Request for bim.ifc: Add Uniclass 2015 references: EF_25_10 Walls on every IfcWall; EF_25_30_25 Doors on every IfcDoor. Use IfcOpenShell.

First a look at what the model holds.

```python
import ifcopenshell

model = ifcopenshell.open("bim.ifc")
print(model.schema)
print("classifications:", [c.Name for c in model.by_type("IfcClassification")])
for ifc_class in ("IfcDoor", "IfcRoof", "IfcStair", "IfcWall", "IfcWindow"):
    print(ifc_class, len(model.by_type(ifc_class)))
```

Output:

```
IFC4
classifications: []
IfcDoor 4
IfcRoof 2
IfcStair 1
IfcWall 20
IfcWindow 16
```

```python
import ifcopenshell
import ifcopenshell.api.classification

model = ifcopenshell.open("bim.ifc")

system = ifcopenshell.api.classification.add_classification(model, classification="Uniclass 2015")

codes = {
    "IfcWall": ("EF_25_10", "Walls"),
    "IfcDoor": ("EF_25_30_25", "Doors"),
}
for ifc_class, (code, name) in codes.items():
    products = model.by_type(ifc_class)
    ifcopenshell.api.classification.add_reference(
        model, products=products, classification=system, identification=code, name=name
    )
    print(code, len(products))

model.write("bim_v2.ifc")
```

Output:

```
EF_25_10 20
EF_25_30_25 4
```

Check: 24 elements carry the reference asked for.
